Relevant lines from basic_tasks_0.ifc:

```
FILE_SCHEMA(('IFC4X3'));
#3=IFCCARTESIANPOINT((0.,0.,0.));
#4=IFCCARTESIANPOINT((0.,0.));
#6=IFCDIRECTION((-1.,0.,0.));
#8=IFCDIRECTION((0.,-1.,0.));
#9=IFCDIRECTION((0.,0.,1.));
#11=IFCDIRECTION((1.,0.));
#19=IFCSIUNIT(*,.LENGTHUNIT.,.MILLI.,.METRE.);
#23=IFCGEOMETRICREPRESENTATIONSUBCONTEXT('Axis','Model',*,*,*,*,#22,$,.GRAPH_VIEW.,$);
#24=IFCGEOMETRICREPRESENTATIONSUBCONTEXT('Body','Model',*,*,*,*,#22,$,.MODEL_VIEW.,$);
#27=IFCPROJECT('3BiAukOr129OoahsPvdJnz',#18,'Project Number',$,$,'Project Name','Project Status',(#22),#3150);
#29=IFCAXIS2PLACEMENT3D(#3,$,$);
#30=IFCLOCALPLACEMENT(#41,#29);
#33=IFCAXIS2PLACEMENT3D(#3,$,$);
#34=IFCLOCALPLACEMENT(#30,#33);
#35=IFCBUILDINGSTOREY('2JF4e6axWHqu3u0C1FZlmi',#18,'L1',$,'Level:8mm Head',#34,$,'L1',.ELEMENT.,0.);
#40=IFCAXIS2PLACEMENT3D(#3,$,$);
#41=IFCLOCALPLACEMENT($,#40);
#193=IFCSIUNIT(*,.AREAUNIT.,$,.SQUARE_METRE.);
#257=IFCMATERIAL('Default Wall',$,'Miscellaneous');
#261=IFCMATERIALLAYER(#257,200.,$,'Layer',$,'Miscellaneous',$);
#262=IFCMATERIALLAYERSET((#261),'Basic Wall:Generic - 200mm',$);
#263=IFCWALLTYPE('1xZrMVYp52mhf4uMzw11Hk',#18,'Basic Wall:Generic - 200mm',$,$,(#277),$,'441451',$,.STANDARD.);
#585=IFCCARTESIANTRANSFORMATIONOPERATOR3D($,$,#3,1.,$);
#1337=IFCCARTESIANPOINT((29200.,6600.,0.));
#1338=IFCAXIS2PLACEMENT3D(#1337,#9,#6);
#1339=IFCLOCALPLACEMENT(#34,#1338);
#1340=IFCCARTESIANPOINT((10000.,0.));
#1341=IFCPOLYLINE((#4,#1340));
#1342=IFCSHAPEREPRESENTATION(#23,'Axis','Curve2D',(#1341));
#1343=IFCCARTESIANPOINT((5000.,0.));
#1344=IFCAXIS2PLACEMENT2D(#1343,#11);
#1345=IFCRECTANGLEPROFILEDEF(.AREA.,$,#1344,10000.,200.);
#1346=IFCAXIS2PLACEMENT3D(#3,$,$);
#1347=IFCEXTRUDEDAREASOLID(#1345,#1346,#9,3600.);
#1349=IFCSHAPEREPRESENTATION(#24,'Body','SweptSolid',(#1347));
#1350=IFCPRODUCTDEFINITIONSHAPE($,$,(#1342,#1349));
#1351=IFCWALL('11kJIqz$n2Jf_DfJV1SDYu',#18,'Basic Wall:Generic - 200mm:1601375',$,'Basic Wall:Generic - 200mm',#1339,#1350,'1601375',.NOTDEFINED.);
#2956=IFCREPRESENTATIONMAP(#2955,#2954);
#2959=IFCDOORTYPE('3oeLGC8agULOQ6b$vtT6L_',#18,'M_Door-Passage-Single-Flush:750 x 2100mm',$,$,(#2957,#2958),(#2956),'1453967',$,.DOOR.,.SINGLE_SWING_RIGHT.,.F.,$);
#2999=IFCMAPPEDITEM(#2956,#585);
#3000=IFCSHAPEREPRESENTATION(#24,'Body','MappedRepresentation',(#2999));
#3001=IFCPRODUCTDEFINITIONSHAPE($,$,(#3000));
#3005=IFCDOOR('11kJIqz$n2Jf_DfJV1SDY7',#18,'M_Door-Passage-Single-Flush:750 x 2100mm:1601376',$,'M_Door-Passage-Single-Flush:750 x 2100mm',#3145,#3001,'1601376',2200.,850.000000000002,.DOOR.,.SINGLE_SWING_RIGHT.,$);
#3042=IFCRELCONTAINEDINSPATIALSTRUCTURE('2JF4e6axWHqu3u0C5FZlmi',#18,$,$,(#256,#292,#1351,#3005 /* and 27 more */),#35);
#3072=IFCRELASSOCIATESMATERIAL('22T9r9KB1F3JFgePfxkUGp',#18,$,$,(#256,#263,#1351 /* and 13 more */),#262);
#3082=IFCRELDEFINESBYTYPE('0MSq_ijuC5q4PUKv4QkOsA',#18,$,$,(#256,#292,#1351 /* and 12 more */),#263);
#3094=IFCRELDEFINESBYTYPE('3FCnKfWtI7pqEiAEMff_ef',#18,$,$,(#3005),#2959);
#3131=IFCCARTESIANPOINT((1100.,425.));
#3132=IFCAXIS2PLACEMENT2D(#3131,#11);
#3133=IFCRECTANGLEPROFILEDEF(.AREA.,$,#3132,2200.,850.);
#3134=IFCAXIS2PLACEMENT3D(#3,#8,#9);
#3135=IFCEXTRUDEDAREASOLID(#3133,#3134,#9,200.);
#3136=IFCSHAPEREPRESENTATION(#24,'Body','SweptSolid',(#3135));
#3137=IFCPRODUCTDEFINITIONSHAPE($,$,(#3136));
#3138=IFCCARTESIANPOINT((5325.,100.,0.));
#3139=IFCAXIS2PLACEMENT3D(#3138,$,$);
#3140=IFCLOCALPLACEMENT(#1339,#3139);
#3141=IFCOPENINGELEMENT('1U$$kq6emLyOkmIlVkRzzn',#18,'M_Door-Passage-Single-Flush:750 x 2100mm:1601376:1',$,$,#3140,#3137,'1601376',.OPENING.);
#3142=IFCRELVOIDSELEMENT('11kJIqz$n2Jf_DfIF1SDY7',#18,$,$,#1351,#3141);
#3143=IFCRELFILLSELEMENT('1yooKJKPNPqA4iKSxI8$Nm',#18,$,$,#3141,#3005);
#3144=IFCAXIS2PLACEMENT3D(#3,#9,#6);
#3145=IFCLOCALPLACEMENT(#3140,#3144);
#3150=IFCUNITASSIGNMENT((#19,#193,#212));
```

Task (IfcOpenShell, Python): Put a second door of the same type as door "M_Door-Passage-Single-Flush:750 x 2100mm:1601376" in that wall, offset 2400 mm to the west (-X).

```python
import ifcopenshell
import ifcopenshell.api.feature
import ifcopenshell.api.geometry
import ifcopenshell.api.root
import ifcopenshell.geom
import ifcopenshell.util.element
import ifcopenshell.util.placement
import ifcopenshell.util.shape

model = ifcopenshell.open("basic_tasks_0.ifc")
settings = ifcopenshell.geom.settings()


def volume(element):
    """Net volume in cubic metres, openings subtracted."""
    shape = ifcopenshell.geom.create_shape(settings, element)
    return ifcopenshell.util.shape.get_volume(shape.geometry)


def reuse_history(source, copy):
    """copy_class also copies each property set's owner history, people and application; keep the originals."""
    for rel in copy.IsDefinedBy:
        if rel.is_a("IfcRelDefinesByProperties") and (history := rel.RelatingPropertyDefinition.OwnerHistory):
            rel.RelatingPropertyDefinition.OwnerHistory = source.OwnerHistory
            ifcopenshell.util.element.remove_deep2(model, history)


door = model.by_guid("11kJIqz$n2Jf_DfJV1SDY7")
opening = door.FillsVoids[0].RelatingOpeningElement
wall = opening.VoidsElements[0].RelatingBuildingElement
before = volume(wall)
shift = ifcopenshell.util.placement.get_local_placement(wall.ObjectPlacement)[:3, 0] * 2400.0

# copy_class copies the void relationship, type, container and properties, but no geometry.
new_opening = ifcopenshell.api.root.copy_class(model, product=opening)
new_opening.Representation = ifcopenshell.util.element.copy_deep(
    model, opening.Representation, exclude=["IfcGeometricRepresentationContext", "IfcRepresentationMap"]
)
new_opening.Name = "M_Door-Passage-Single-Flush:750 x 2100mm"
new_opening.Tag = None
new_door = ifcopenshell.api.root.copy_class(model, product=door)
new_door.Representation = ifcopenshell.util.element.copy_deep(
    model, door.Representation, exclude=["IfcGeometricRepresentationContext", "IfcRepresentationMap"]
)
new_door.Name = "M_Door-Passage-Single-Flush:750 x 2100mm"
new_door.Tag = None
reuse_history(door, new_door)
ifcopenshell.api.feature.add_filling(model, opening=new_opening, element=new_door)

for old, new in ((opening, new_opening), (door, new_door)):
    matrix = ifcopenshell.util.placement.get_local_placement(old.ObjectPlacement)
    matrix[:3, 3] += shift
    ifcopenshell.api.geometry.edit_object_placement(model, product=new, matrix=matrix, is_si=False)

after = volume(wall)

print(f"wall volume {before:.3f} -> {after:.3f} m3")

model.write("basic_tasks_0_rev.ifc")
```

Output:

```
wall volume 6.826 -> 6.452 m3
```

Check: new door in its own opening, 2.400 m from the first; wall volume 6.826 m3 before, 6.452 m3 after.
